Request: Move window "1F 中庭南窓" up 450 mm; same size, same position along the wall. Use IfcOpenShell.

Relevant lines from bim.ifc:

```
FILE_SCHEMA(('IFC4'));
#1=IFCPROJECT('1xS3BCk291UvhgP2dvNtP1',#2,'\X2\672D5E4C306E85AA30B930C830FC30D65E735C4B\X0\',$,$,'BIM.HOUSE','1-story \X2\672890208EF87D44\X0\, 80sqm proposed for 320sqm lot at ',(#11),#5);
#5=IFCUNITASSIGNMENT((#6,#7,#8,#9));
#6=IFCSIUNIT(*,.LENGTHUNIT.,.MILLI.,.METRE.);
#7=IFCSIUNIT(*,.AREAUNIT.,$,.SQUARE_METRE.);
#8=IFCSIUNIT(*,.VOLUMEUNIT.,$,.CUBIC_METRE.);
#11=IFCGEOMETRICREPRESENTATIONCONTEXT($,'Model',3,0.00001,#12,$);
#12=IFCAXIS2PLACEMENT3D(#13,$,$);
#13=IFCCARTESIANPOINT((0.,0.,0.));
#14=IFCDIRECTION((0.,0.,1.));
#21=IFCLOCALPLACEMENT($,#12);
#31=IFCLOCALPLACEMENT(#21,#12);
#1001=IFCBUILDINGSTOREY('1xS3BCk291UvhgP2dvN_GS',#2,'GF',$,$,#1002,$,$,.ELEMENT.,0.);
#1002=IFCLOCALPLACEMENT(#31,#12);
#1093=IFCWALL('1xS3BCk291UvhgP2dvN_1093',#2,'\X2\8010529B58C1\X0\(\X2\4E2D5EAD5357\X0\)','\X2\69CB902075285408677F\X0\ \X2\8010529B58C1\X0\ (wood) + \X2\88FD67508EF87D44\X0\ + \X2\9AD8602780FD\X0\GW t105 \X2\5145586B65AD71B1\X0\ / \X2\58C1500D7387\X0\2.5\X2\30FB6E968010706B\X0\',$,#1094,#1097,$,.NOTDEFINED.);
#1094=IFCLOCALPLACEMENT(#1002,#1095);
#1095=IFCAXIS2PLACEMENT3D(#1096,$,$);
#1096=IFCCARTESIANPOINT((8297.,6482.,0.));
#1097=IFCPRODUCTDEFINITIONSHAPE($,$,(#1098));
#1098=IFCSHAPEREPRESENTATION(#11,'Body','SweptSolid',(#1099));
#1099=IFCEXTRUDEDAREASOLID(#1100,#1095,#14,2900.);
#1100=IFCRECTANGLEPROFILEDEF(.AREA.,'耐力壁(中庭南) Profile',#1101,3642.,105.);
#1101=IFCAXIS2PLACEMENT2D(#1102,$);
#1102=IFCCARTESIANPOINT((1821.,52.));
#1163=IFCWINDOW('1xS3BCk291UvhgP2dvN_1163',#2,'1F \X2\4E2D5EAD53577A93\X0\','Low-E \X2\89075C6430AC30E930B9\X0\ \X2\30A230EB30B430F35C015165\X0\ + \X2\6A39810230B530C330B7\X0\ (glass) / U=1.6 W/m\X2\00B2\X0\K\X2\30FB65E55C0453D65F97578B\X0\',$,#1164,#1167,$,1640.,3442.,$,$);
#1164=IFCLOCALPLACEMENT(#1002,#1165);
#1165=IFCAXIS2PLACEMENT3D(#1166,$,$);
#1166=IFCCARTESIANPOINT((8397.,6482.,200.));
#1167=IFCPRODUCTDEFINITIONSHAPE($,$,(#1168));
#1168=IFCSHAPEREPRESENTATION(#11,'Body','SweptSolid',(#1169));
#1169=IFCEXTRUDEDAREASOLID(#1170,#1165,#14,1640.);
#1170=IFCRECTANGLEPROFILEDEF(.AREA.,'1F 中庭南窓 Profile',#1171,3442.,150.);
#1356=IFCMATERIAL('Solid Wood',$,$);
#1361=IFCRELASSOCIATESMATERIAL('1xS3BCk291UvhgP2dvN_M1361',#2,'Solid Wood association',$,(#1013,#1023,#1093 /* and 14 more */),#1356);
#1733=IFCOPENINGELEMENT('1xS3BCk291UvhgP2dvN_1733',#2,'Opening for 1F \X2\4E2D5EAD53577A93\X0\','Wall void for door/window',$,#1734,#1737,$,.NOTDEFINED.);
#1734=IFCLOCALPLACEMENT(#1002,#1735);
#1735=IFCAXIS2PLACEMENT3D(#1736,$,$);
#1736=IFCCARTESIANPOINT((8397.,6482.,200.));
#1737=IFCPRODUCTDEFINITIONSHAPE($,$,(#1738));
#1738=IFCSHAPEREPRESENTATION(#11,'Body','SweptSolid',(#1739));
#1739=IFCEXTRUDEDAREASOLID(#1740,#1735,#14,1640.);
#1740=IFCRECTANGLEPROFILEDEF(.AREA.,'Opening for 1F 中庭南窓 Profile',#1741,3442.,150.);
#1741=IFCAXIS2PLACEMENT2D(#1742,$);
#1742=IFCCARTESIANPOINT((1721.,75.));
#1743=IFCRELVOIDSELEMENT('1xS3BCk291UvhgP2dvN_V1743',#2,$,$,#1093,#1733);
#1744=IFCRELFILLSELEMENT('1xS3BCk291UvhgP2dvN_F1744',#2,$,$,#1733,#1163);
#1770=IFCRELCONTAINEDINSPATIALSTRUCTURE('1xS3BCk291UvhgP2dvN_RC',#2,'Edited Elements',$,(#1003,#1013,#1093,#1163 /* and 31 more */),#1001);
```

```python
import numpy as np
import ifcopenshell
import ifcopenshell.api.geometry
import ifcopenshell.util.placement
import ifcopenshell.util.unit

model = ifcopenshell.open("bim.ifc")
unit_scale = ifcopenshell.util.unit.calculate_unit_scale(model)

window = model.by_guid("1xS3BCk291UvhgP2dvN_1163")
opening = window.FillsVoids[0].RelatingOpeningElement
dz = 0.45 / unit_scale

shift = np.array([0.0, 0.0, dz])
# The window is not placed relative to its opening, so move both.
for product in (opening, window):
    matrix = ifcopenshell.util.placement.get_local_placement(product.ObjectPlacement)
    matrix[:3, 3] += shift
    ifcopenshell.api.geometry.edit_object_placement(model, product=product, matrix=matrix, is_si=False)

print(f"moved by {dz * unit_scale:+.3f} m")

model.write("bim_updated.ifc")
```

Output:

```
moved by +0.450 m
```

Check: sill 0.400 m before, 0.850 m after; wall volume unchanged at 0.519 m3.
